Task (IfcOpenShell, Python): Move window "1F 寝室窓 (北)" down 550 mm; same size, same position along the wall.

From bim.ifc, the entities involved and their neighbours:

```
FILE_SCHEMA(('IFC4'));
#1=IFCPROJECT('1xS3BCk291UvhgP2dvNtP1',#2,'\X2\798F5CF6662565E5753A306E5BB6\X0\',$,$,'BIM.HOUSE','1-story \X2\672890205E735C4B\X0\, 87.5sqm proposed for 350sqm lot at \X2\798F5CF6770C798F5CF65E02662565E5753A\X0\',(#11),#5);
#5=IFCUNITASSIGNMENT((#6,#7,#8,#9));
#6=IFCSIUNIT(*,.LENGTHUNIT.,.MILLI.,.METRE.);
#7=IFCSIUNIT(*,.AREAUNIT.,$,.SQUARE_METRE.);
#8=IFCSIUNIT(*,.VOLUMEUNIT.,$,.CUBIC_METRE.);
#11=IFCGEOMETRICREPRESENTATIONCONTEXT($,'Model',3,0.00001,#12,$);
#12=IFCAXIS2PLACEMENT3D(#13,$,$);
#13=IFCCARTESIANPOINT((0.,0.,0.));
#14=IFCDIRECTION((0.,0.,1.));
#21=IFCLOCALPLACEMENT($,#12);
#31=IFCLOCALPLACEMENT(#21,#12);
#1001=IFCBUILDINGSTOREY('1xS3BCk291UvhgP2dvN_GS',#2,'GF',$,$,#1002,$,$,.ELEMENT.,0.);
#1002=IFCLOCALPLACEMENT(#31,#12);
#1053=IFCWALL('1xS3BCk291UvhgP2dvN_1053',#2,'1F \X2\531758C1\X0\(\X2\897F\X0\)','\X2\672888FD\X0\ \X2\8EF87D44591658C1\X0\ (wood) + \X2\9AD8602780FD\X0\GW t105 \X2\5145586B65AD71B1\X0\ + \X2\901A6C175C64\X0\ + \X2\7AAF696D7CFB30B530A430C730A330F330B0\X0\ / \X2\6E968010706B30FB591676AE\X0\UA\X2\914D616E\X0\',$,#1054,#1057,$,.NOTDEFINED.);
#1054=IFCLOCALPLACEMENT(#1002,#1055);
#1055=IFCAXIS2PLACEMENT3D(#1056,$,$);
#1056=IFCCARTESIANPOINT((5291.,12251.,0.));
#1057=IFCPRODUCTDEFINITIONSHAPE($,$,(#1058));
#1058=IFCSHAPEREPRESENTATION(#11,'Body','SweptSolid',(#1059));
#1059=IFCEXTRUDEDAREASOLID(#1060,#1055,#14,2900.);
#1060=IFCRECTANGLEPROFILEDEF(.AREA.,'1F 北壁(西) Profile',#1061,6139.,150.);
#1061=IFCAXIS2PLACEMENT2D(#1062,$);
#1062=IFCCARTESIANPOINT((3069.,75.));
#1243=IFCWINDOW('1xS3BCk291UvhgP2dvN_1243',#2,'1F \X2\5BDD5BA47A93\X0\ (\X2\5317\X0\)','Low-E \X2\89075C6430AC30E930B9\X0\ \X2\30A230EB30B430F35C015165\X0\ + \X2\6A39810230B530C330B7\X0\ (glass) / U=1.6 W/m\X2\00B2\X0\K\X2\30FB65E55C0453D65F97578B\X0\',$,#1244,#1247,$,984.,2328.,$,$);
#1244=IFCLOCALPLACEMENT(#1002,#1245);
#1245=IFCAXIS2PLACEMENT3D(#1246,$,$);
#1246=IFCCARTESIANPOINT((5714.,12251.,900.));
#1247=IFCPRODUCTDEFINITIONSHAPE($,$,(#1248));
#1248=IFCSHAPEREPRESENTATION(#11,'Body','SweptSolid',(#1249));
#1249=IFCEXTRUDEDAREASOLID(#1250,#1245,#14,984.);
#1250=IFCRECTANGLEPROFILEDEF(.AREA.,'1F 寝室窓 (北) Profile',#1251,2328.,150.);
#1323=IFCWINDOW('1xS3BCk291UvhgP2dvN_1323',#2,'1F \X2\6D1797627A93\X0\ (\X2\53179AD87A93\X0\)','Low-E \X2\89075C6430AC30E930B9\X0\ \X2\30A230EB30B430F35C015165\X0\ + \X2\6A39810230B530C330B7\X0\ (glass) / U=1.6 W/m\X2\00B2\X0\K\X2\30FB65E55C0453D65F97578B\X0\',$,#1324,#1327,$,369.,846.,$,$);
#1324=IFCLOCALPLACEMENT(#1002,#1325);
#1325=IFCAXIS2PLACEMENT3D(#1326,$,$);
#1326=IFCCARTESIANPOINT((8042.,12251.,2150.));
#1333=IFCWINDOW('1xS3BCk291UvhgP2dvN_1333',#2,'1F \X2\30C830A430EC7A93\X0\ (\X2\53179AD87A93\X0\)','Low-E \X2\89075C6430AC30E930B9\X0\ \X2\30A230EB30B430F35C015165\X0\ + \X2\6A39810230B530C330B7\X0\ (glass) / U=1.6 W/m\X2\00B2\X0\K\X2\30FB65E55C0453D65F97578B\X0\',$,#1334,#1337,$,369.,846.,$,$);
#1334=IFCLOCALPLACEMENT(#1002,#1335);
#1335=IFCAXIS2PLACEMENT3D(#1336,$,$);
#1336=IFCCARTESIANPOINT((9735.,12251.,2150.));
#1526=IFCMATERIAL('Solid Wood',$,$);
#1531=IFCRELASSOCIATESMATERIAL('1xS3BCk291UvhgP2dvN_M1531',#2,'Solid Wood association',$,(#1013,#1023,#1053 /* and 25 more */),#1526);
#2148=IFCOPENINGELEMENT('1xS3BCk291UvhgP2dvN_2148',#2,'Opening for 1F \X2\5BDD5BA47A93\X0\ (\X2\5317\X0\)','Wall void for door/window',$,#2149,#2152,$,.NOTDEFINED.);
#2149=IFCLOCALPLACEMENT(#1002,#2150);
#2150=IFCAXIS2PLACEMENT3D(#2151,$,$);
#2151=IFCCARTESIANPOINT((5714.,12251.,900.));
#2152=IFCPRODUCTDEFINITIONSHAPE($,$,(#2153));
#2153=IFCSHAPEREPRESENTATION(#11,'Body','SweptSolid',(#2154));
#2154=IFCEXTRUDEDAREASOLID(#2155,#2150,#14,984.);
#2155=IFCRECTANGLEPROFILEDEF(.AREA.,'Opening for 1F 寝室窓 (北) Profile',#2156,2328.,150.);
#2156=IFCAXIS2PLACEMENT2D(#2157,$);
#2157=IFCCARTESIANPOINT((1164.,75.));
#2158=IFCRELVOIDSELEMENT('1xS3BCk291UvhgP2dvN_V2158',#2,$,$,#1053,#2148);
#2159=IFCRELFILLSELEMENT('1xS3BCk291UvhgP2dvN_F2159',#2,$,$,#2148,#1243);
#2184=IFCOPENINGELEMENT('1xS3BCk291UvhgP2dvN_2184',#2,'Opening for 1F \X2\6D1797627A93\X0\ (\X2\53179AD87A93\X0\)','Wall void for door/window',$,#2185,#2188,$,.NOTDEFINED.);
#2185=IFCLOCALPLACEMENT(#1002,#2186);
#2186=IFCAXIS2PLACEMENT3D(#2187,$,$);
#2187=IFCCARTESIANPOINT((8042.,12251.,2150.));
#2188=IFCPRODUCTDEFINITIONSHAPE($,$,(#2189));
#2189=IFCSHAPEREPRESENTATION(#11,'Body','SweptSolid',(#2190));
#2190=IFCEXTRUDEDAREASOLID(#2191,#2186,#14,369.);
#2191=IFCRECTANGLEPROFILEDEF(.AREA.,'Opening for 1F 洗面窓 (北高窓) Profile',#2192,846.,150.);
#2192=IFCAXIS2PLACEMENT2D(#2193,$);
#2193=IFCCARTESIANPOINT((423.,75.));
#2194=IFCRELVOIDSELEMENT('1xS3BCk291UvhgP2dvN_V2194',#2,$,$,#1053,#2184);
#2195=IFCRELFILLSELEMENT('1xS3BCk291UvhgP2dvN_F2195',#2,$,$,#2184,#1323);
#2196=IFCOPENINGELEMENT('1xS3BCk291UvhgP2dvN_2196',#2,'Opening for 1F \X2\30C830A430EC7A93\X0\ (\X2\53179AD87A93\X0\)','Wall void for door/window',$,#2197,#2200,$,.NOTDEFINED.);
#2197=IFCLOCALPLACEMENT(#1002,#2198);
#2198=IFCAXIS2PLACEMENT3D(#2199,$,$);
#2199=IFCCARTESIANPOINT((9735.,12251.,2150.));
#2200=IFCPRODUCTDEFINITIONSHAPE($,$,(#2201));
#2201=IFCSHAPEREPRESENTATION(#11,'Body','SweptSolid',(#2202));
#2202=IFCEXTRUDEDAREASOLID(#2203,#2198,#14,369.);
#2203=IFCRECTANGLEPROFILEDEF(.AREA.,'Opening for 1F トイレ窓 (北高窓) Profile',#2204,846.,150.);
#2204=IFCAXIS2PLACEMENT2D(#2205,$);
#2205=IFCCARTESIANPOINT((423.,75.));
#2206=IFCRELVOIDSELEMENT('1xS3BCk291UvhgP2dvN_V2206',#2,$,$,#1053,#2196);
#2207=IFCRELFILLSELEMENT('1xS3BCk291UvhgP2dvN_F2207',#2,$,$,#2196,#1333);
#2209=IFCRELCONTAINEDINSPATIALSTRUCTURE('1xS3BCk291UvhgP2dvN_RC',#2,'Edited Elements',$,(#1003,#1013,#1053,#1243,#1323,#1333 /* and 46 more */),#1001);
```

```python
import numpy as np
import ifcopenshell
import ifcopenshell.api.geometry
import ifcopenshell.util.placement
import ifcopenshell.util.unit

model = ifcopenshell.open("bim.ifc")
unit_scale = ifcopenshell.util.unit.calculate_unit_scale(model)

window = model.by_id(1243)
opening = window.FillsVoids[0].RelatingOpeningElement
dz = -0.55 / unit_scale

shift = np.array([0.0, 0.0, dz])
# The window is not placed relative to its opening, so move both.
for product in (opening, window):
    matrix = ifcopenshell.util.placement.get_local_placement(product.ObjectPlacement)
    matrix[:3, 3] += shift
    ifcopenshell.api.geometry.edit_object_placement(model, product=product, matrix=matrix, is_si=False)

print(f"moved by {dz * unit_scale:+.3f} m")

model.write("bim_v2.ifc")
```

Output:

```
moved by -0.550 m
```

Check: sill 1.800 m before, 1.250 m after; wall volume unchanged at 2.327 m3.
